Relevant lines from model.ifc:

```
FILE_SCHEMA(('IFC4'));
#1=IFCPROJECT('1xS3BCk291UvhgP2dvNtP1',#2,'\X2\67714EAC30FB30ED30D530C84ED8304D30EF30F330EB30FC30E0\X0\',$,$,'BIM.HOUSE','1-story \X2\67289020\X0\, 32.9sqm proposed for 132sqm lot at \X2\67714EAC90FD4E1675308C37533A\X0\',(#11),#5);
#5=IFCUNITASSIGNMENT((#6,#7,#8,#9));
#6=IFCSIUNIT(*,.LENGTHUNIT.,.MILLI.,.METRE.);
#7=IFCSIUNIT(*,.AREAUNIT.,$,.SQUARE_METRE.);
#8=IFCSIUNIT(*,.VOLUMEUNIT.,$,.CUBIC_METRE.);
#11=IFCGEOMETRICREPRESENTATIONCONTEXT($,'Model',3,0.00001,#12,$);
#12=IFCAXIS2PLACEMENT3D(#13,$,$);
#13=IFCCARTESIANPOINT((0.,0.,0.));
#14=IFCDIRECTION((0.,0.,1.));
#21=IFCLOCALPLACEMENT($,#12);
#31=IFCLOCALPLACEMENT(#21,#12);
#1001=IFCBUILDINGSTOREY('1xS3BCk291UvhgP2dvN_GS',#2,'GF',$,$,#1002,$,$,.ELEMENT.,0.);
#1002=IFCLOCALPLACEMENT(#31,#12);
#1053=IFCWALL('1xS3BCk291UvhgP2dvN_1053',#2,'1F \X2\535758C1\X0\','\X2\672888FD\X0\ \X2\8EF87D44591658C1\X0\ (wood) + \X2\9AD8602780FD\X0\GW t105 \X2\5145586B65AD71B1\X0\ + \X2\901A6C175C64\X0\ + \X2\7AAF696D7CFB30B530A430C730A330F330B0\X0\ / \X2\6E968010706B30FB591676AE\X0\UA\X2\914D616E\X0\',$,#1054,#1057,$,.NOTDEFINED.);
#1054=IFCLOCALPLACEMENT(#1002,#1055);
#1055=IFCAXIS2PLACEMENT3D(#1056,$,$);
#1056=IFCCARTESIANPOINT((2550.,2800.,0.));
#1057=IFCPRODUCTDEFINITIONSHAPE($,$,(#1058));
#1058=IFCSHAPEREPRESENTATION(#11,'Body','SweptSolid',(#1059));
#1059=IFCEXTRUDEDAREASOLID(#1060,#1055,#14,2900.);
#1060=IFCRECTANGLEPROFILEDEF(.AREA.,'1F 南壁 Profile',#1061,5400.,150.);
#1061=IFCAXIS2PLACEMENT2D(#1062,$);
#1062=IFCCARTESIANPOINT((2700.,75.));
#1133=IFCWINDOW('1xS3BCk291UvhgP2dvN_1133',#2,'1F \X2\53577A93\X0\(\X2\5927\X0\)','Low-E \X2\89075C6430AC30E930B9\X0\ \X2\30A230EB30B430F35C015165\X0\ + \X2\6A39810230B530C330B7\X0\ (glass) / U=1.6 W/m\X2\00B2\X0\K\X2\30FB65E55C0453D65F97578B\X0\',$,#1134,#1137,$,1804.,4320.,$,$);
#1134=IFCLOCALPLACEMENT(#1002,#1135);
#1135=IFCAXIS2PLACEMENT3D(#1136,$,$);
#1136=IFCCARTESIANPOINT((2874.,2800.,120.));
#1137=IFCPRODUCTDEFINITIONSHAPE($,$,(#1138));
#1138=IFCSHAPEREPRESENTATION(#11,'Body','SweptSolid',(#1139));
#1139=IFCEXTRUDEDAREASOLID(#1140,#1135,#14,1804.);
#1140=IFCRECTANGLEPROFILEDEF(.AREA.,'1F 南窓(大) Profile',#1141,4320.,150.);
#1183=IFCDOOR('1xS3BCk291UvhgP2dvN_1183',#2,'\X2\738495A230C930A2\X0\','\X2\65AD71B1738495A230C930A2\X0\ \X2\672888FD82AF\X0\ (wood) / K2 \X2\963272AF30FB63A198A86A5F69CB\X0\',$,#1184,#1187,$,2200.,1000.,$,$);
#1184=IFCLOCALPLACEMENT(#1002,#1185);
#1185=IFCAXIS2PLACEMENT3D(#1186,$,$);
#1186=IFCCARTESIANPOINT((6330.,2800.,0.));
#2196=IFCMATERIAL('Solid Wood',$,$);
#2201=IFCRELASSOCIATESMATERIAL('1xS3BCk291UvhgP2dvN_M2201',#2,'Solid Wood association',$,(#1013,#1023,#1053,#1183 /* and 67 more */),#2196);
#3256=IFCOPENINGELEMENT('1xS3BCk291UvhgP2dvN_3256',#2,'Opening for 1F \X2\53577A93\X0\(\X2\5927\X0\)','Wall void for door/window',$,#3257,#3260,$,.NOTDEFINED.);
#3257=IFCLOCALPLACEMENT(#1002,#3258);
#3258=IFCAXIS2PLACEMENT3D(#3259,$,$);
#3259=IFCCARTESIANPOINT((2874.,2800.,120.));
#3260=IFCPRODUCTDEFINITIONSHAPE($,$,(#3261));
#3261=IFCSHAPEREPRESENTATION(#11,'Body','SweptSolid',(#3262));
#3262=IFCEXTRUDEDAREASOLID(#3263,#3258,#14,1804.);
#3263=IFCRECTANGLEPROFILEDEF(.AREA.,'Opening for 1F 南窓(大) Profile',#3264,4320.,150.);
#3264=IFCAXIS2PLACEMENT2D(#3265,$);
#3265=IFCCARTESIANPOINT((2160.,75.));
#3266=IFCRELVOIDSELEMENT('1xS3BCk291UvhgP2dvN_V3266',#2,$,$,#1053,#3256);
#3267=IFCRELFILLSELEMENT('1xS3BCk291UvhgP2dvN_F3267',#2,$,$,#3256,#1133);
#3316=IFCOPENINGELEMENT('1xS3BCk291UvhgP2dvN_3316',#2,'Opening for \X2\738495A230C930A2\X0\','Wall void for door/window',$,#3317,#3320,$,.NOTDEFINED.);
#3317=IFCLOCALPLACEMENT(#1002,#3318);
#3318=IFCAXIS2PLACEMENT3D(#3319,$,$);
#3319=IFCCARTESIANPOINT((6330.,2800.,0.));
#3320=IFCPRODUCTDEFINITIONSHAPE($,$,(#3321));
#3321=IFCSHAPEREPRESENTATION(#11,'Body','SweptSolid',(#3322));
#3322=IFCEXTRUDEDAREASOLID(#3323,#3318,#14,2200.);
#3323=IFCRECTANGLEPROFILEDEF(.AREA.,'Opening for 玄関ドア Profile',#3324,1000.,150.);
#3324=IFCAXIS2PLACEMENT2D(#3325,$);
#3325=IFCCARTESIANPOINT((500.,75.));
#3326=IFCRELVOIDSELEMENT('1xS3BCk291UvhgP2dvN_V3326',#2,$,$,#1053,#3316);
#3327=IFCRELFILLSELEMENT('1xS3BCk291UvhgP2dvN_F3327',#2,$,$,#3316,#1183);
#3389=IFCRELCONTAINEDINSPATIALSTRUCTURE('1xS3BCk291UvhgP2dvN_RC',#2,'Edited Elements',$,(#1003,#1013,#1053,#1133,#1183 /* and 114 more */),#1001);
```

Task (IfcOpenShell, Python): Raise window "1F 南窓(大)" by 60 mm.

```python
import numpy as np
import ifcopenshell
import ifcopenshell.api.geometry
import ifcopenshell.util.placement
import ifcopenshell.util.unit

model = ifcopenshell.open("model.ifc")
unit_scale = ifcopenshell.util.unit.calculate_unit_scale(model)

window = model.by_guid("1xS3BCk291UvhgP2dvN_1133")
opening = window.FillsVoids[0].RelatingOpeningElement
dz = 0.06 / unit_scale

shift = np.array([0.0, 0.0, dz])
# The window is not placed relative to its opening, so move both.
for product in (opening, window):
    matrix = ifcopenshell.util.placement.get_local_placement(product.ObjectPlacement)
    matrix[:3, 3] += shift
    ifcopenshell.api.geometry.edit_object_placement(model, product=product, matrix=matrix, is_si=False)

print(f"moved by {dz * unit_scale:+.3f} m")

model.write("model_rev.ifc")
```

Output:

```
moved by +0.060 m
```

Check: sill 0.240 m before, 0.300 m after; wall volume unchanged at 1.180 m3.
